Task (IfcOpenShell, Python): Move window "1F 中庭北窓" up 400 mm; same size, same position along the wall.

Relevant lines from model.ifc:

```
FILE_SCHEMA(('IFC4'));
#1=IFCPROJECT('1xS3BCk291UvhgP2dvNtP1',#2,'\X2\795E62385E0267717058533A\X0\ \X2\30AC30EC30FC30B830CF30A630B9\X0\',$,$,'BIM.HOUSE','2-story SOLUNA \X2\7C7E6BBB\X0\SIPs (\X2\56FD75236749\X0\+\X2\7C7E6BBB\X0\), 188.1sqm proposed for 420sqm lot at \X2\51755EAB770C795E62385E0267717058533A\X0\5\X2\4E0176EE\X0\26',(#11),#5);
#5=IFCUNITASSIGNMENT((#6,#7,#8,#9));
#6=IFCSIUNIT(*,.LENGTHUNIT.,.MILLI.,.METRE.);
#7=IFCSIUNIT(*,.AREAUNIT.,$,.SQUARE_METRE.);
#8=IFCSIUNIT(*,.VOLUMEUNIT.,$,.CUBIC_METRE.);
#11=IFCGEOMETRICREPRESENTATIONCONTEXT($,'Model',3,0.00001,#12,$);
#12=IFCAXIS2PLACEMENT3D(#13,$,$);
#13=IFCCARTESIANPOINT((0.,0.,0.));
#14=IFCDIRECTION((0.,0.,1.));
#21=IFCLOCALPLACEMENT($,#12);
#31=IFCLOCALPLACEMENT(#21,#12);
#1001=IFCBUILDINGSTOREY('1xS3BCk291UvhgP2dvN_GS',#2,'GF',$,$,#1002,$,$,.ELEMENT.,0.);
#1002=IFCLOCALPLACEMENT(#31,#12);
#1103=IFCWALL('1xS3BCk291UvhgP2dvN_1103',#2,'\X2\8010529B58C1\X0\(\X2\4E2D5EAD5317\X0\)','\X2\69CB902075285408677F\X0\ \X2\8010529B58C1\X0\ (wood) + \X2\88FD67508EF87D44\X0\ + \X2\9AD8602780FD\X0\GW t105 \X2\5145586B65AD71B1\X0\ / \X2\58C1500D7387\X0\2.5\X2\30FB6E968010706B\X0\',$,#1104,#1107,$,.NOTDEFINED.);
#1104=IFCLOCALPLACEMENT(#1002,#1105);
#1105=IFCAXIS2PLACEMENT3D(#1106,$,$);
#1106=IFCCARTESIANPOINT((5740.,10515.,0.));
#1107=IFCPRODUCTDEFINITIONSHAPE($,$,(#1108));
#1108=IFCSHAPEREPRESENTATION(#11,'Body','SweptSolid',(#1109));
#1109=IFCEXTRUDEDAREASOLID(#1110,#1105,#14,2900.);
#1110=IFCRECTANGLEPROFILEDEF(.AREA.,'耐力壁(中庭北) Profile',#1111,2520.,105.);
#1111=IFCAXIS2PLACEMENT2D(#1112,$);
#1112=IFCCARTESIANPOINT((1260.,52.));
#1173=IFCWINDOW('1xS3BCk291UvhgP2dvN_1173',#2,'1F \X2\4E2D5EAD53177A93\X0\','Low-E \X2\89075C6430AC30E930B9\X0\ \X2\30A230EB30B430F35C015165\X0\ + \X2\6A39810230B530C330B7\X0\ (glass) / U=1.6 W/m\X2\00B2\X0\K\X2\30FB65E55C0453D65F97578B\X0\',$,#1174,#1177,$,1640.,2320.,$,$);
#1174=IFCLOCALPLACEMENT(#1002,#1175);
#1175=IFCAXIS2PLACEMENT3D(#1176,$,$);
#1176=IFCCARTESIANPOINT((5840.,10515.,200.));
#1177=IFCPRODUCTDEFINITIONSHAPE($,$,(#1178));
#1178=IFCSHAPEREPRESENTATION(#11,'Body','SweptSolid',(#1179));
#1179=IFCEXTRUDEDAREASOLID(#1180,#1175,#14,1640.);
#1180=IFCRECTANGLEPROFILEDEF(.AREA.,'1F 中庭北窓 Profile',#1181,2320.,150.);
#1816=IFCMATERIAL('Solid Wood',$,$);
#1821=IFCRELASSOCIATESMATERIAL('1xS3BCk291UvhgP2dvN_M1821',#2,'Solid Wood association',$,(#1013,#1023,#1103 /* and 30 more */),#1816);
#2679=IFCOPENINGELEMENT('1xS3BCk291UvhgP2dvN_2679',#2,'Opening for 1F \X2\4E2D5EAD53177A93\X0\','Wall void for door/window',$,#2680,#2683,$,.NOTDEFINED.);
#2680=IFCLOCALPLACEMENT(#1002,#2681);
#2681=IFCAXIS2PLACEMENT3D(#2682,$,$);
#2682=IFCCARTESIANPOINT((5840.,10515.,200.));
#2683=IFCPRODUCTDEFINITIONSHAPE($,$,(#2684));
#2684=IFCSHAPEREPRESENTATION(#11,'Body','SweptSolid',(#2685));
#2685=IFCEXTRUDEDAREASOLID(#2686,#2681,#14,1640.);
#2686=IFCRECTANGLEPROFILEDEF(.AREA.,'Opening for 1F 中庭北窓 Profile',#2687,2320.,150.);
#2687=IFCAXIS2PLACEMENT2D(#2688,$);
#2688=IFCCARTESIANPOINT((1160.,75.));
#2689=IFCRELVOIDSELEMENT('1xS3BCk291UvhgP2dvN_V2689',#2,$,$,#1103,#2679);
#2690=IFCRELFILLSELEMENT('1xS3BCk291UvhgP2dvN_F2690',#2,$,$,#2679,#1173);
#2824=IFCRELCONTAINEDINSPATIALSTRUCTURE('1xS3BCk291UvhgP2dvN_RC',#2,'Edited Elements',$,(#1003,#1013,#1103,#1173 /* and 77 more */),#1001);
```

```python
import numpy as np
import ifcopenshell
import ifcopenshell.api.geometry
import ifcopenshell.util.placement
import ifcopenshell.util.unit

model = ifcopenshell.open("model.ifc")
unit_scale = ifcopenshell.util.unit.calculate_unit_scale(model)

window = model.by_id(1173)
opening = window.FillsVoids[0].RelatingOpeningElement
dz = 0.4 / unit_scale

shift = np.array([0.0, 0.0, dz])
# The window is not placed relative to its opening, so move both.
for product in (opening, window):
    matrix = ifcopenshell.util.placement.get_local_placement(product.ObjectPlacement)
    matrix[:3, 3] += shift
    ifcopenshell.api.geometry.edit_object_placement(model, product=product, matrix=matrix, is_si=False)

print(f"moved by {dz * unit_scale:+.3f} m")

model.write("model_updated.ifc")
```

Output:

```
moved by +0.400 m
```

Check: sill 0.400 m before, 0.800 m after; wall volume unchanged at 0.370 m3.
